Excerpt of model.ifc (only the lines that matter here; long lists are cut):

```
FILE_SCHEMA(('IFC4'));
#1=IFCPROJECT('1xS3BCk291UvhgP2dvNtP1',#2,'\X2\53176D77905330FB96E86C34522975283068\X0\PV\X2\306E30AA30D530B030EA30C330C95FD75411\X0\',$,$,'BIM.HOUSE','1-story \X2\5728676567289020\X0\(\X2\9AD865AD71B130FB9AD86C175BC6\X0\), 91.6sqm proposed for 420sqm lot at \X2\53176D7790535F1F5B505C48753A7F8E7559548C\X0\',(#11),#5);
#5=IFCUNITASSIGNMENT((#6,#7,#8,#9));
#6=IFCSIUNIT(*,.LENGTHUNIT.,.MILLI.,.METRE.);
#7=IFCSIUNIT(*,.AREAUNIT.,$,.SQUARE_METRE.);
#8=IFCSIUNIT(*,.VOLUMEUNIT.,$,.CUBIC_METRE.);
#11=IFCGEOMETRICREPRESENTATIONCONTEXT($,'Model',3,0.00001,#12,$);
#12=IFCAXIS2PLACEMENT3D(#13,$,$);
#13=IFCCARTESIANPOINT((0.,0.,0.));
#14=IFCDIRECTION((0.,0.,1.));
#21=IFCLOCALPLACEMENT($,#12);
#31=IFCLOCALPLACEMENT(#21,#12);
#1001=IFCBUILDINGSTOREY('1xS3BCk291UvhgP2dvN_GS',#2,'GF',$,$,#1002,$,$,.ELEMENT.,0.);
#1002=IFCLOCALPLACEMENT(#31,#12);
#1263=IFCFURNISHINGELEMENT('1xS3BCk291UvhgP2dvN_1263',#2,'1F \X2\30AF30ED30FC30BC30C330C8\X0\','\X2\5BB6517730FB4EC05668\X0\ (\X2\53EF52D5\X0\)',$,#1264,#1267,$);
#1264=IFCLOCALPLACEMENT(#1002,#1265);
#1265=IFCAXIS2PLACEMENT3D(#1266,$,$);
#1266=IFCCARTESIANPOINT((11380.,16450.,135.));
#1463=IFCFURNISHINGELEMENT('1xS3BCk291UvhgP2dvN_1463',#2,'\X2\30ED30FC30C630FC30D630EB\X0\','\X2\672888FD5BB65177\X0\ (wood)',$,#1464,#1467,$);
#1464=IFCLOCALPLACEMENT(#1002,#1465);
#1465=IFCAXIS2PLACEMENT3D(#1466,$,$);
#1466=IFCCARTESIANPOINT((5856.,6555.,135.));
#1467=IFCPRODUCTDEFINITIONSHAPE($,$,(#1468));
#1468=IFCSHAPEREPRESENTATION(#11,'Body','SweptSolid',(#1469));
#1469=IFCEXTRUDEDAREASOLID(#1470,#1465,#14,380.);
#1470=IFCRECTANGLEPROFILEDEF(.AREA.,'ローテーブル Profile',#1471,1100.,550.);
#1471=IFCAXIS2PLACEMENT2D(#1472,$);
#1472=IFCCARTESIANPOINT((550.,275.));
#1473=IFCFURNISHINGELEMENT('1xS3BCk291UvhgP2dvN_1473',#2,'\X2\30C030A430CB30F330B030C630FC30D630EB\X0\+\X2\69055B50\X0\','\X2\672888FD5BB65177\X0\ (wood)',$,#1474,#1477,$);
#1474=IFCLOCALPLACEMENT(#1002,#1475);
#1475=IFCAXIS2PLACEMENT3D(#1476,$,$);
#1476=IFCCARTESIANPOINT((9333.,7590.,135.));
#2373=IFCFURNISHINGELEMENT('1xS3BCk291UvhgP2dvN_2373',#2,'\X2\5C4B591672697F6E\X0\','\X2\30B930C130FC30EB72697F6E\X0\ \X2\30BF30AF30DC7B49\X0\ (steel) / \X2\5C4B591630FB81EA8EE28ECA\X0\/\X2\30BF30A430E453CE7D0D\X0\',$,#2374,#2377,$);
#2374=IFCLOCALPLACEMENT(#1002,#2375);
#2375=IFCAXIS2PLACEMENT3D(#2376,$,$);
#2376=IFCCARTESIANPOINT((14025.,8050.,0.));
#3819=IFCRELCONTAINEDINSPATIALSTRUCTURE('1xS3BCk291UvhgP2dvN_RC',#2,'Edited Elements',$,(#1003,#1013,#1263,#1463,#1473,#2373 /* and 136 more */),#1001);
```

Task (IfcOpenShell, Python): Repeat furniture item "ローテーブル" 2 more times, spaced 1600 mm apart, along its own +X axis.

```python
import ifcopenshell
import ifcopenshell.api.geometry
import ifcopenshell.api.root
import ifcopenshell.util.element
import ifcopenshell.util.placement

model = ifcopenshell.open("model.ifc")


def reuse_history(source, copy):
    """copy_class also copies each property set's owner history, people and application; keep the originals."""
    for rel in copy.IsDefinedBy:
        if rel.is_a("IfcRelDefinesByProperties") and (history := rel.RelatingPropertyDefinition.OwnerHistory):
            rel.RelatingPropertyDefinition.OwnerHistory = source.OwnerHistory
            ifcopenshell.util.element.remove_deep2(model, history)


source = model.by_guid("1xS3BCk291UvhgP2dvN_1463")
base = ifcopenshell.util.placement.get_local_placement(source.ObjectPlacement)
step = base[:3, 0] * 1600.0

for i in range(1, 3):
    copy = ifcopenshell.api.root.copy_class(model, product=source)
    copy.Representation = ifcopenshell.util.element.copy_deep(
        model, source.Representation, exclude=["IfcGeometricRepresentationContext", "IfcRepresentationMap"]
    )
    reuse_history(source, copy)
    matrix = base.copy()
    matrix[:3, 3] += i * step
    print("added at", matrix[:3, 3].round(3) + 0.0)
    ifcopenshell.api.geometry.edit_object_placement(model, product=copy, matrix=matrix, is_si=False)

model.write("model_rev.ifc")
```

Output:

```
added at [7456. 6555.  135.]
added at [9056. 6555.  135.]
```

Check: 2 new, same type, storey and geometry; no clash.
